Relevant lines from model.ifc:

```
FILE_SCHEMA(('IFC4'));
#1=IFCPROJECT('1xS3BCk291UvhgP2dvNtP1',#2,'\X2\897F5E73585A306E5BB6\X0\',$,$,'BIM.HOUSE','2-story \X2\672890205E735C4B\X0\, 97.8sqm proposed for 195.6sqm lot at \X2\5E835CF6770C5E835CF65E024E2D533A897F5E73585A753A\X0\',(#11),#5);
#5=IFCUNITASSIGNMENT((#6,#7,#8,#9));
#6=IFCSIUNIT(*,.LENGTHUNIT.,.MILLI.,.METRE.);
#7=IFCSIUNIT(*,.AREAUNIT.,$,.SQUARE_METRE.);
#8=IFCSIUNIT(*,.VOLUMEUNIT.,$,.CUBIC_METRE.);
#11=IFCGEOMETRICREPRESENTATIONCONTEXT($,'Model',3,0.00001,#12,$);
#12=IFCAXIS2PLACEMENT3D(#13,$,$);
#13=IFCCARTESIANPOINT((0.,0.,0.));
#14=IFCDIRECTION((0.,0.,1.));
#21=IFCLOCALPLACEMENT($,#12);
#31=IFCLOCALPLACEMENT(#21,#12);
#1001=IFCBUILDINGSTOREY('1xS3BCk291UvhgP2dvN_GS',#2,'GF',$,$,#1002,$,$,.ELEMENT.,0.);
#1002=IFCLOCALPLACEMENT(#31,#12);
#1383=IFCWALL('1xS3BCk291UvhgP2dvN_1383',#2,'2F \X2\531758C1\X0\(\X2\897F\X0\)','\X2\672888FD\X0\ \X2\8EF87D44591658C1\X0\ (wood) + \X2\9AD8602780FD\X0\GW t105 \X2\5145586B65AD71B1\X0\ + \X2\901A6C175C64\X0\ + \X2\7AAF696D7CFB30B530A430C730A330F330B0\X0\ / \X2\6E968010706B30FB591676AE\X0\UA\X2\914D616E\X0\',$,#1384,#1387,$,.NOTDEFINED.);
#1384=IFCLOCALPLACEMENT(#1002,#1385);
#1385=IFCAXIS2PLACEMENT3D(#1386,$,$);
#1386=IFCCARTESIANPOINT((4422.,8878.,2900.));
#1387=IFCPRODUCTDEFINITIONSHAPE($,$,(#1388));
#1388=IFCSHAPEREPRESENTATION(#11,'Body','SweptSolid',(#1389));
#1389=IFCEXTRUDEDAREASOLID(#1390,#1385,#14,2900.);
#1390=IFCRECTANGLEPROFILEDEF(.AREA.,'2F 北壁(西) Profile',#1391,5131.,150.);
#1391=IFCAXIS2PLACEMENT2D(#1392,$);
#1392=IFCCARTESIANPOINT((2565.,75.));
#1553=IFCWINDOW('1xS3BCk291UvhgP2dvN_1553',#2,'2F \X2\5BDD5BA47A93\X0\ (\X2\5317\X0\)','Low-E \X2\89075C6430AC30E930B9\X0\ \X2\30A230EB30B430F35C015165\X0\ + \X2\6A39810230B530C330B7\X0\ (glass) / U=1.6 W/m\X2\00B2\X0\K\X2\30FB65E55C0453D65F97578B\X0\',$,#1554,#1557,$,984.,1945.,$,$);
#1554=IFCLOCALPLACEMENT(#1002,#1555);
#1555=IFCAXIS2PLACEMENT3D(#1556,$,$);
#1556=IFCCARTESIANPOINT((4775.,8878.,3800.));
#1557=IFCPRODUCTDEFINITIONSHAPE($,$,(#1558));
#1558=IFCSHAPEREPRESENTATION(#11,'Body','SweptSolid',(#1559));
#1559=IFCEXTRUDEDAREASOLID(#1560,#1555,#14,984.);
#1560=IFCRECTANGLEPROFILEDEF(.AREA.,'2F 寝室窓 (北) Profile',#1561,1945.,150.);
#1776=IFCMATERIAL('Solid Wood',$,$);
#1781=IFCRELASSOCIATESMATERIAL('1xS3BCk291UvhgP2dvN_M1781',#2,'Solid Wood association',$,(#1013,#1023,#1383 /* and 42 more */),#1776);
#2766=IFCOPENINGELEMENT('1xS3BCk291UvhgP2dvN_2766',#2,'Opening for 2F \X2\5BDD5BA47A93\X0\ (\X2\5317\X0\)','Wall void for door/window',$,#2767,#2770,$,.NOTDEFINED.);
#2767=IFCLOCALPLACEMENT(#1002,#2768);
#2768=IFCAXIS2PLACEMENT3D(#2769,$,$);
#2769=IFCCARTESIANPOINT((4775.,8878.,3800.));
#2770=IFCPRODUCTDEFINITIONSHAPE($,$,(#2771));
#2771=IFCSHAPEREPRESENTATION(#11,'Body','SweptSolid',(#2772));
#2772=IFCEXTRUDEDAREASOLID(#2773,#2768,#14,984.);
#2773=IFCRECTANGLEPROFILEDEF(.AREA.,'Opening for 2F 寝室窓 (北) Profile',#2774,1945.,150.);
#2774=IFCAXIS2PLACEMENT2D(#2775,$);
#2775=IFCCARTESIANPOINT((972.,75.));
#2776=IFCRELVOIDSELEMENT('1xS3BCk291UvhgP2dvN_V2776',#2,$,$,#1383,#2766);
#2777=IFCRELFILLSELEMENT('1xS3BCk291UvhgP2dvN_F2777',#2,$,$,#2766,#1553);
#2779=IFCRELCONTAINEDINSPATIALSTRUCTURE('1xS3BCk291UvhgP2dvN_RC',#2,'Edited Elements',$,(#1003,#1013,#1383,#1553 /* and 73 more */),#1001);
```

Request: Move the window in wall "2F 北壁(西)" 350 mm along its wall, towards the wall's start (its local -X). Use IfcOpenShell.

```python
import ifcopenshell
import ifcopenshell.api.geometry
import ifcopenshell.util.placement

model = ifcopenshell.open("model.ifc")

window = model.by_id(1553)
opening = window.FillsVoids[0].RelatingOpeningElement
wall = opening.VoidsElements[0].RelatingBuildingElement

wall_matrix = ifcopenshell.util.placement.get_local_placement(wall.ObjectPlacement)
shift = wall_matrix[:3, 0] * -350.0
before = ifcopenshell.util.placement.get_local_placement(window.ObjectPlacement)[:3, 3].copy()

# The window is not placed relative to its opening, so move both.
for product in (opening, window):
    matrix = ifcopenshell.util.placement.get_local_placement(product.ObjectPlacement)
    matrix[:3, 3] += shift
    ifcopenshell.api.geometry.edit_object_placement(model, product=product, matrix=matrix, is_si=False)

after = ifcopenshell.util.placement.get_local_placement(window.ObjectPlacement)[:3, 3]
print("window moved by", (after - before).round(3) + 0.0)

model.write("model_v2.ifc")
```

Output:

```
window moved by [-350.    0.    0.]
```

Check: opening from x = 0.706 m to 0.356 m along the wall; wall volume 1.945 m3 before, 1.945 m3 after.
